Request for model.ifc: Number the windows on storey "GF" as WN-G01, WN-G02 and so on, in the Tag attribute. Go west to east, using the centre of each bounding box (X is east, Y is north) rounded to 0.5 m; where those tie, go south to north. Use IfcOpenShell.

First a look at what the model holds.

```python
import ifcopenshell
import ifcopenshell.util.element
import ifcopenshell.util.placement

model = ifcopenshell.open("model.ifc")
print(model.schema)
storey = next(s for s in model.by_type("IfcBuildingStorey") if s.Name == "GF")
windows = [e for e in ifcopenshell.util.element.get_decomposition(storey) if e.is_a("IfcWindow")]
for e in sorted(windows, key=lambda e: e.id()):
    origin = ifcopenshell.util.placement.get_local_placement(e.ObjectPlacement)[:3, 3]
    print(e.id(), e.Tag, e.Name, origin.round(2) + 0.0, sep=" | ")
```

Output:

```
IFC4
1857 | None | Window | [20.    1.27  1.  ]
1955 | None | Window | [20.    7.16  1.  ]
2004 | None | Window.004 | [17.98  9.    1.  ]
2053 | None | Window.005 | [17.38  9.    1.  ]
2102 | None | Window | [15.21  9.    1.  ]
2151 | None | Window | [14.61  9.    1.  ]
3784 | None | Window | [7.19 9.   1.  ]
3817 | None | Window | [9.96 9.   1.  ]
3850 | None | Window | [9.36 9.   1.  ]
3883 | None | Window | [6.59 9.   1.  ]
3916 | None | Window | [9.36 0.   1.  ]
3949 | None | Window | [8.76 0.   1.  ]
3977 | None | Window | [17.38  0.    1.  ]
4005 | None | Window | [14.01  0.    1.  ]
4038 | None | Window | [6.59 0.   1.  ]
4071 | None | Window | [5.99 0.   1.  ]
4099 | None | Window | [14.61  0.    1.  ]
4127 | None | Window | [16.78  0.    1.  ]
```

```python
import ifcopenshell
import ifcopenshell.geom
import ifcopenshell.util.element
import ifcopenshell.util.shape

model = ifcopenshell.open("model.ifc")
settings = ifcopenshell.geom.settings()
settings.set("use-world-coords", True)


def centre(element):
    shape = ifcopenshell.geom.create_shape(settings, element)
    return ifcopenshell.util.shape.get_bbox_centroid(shape.geometry)


storey = next(s for s in model.by_type("IfcBuildingStorey") if s.Name == "GF")
windows = [e for e in ifcopenshell.util.element.get_decomposition(storey) if e.is_a("IfcWindow")]

# Insertion points can sit at a corner or the storey origin, so sort by the geometry (in metres).
centres = {e: centre(e) for e in windows}
windows.sort(key=lambda e: (round(centres[e][0] / 0.5), centres[e][1]))

for i, e in enumerate(windows, start=1):
    number = f"WN-G{i:02d}"
    e.Tag = number
    print(e.id(), number)

model.write("model-out.ifc")
```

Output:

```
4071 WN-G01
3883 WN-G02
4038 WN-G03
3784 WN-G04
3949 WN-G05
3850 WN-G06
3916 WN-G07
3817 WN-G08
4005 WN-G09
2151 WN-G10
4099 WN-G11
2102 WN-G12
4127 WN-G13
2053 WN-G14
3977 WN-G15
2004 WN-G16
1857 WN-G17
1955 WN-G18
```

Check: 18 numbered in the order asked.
